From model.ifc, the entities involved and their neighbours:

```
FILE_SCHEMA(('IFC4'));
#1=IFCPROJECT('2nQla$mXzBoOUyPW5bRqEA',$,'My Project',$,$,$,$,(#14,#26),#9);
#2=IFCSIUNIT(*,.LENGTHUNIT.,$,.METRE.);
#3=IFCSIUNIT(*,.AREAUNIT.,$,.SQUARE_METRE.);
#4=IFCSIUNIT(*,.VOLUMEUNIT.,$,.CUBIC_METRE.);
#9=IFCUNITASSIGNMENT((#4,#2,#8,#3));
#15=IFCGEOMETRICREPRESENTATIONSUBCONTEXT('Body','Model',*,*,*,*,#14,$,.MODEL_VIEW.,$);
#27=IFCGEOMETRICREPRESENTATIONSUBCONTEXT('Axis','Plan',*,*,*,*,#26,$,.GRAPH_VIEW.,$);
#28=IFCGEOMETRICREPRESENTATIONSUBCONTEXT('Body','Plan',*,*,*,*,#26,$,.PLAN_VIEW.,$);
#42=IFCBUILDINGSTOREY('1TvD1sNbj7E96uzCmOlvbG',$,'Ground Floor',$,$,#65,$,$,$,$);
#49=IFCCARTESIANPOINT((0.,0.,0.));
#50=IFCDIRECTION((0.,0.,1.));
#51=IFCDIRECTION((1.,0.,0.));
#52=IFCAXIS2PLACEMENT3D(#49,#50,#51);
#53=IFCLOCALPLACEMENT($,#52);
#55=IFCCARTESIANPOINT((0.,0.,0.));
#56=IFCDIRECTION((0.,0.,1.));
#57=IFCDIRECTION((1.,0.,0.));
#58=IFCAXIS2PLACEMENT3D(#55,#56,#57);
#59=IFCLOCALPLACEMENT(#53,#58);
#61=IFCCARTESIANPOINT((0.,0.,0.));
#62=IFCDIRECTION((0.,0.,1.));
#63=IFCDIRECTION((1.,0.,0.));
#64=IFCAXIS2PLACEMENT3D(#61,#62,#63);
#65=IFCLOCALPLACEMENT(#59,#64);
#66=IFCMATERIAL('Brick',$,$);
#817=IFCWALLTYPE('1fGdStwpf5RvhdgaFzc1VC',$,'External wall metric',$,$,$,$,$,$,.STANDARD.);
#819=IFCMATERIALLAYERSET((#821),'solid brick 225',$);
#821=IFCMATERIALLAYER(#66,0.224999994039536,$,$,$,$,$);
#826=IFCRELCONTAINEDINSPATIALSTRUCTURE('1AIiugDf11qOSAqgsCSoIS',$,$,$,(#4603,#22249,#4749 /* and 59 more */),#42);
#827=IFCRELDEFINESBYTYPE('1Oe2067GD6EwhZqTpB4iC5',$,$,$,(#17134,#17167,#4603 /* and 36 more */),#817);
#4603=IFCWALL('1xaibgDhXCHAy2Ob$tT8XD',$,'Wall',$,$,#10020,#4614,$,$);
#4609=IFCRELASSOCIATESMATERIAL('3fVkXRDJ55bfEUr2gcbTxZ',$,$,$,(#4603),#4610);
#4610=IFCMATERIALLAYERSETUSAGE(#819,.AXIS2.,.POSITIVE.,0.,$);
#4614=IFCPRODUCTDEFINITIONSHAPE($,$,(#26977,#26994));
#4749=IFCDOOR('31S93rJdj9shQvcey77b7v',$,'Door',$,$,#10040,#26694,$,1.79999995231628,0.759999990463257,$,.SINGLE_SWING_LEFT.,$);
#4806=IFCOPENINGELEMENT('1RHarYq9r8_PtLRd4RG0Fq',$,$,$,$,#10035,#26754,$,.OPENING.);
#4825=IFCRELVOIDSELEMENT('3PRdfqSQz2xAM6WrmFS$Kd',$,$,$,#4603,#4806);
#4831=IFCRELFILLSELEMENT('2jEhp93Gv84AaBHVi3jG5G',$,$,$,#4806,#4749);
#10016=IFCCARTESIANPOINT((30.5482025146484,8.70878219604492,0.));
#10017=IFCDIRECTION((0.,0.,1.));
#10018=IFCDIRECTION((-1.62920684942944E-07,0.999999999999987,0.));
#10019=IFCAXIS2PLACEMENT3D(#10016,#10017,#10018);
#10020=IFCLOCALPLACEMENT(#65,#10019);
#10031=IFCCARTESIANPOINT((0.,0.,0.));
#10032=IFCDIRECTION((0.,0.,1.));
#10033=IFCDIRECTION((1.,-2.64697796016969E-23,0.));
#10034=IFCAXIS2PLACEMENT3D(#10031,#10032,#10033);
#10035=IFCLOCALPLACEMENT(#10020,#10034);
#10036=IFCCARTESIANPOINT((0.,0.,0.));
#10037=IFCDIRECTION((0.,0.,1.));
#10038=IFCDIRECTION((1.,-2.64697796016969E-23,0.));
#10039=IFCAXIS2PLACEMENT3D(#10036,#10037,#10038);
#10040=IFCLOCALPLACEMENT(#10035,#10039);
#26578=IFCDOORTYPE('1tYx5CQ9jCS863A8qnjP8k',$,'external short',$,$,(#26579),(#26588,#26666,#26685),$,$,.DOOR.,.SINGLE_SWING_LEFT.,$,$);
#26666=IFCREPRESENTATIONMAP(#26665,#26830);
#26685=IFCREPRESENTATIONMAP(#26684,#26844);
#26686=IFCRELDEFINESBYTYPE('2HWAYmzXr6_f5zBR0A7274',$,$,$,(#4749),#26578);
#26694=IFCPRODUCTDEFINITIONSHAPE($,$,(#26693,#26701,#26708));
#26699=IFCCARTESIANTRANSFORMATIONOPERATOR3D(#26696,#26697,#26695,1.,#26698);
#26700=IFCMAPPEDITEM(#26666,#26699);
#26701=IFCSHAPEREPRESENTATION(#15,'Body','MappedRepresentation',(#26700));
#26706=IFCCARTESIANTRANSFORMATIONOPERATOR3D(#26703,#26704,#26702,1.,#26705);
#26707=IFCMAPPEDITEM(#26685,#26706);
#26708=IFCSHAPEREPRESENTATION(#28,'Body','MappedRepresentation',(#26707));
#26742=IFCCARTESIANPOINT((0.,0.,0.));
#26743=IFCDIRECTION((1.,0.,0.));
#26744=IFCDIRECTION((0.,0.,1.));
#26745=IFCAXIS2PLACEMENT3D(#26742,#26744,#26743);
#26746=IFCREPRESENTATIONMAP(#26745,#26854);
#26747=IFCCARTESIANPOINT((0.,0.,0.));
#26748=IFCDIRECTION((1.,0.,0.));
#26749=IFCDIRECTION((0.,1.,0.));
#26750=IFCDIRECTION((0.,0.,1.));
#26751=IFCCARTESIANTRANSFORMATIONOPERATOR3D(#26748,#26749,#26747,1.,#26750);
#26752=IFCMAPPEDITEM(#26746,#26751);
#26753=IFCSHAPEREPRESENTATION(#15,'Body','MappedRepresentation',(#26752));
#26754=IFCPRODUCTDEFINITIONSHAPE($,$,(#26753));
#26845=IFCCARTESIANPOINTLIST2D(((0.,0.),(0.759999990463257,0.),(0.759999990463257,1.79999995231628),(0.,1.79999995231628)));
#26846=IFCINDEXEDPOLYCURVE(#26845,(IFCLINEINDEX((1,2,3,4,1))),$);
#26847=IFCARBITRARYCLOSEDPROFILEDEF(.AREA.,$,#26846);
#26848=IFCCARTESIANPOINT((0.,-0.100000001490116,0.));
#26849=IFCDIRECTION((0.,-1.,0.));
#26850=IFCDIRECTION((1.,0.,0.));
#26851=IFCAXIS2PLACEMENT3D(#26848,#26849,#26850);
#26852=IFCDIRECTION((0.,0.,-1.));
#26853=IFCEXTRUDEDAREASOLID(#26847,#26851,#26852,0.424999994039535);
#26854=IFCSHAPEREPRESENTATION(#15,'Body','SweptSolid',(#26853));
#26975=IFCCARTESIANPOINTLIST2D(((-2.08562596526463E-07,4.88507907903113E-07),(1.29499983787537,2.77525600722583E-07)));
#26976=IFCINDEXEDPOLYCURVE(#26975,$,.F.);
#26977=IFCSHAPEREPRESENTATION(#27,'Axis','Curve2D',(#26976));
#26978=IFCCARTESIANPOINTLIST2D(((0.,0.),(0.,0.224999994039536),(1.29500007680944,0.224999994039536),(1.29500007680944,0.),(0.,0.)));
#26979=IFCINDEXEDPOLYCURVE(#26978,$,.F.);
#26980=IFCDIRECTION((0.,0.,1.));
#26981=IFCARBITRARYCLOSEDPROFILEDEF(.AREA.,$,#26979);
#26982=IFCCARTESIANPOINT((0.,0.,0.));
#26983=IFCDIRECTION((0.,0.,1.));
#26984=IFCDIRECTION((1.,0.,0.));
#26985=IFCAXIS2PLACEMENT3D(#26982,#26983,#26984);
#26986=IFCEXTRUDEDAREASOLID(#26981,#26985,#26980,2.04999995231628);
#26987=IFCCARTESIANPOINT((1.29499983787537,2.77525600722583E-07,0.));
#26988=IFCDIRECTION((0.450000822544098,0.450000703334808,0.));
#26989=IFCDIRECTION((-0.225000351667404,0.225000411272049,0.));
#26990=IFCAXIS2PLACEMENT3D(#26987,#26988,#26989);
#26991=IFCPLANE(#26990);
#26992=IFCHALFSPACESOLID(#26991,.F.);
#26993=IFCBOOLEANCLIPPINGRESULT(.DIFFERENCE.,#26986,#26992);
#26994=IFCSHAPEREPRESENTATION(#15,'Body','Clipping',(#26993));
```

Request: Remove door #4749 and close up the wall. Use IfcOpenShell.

```python
import ifcopenshell
import ifcopenshell.api.feature
import ifcopenshell.api.root
import ifcopenshell.geom
import ifcopenshell.util.shape

model = ifcopenshell.open("model.ifc")
settings = ifcopenshell.geom.settings()


def volume(element):
    """Net volume in cubic metres, openings subtracted."""
    shape = ifcopenshell.geom.create_shape(settings, element)
    return ifcopenshell.util.shape.get_volume(shape.geometry)


door = model.by_guid("31S93rJdj9shQvcey77b7v")
opening = door.FillsVoids[0].RelatingOpeningElement
wall = opening.VoidsElements[0].RelatingBuildingElement
before = volume(wall)

ifcopenshell.api.root.remove_product(model, product=door)
ifcopenshell.api.feature.remove_feature(model, feature=opening)

after = volume(wall)

print(f"wall volume {before:.3f} -> {after:.3f} m3")

model.write("model_updated.ifc")
```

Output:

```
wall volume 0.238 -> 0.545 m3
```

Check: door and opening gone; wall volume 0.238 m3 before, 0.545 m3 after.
